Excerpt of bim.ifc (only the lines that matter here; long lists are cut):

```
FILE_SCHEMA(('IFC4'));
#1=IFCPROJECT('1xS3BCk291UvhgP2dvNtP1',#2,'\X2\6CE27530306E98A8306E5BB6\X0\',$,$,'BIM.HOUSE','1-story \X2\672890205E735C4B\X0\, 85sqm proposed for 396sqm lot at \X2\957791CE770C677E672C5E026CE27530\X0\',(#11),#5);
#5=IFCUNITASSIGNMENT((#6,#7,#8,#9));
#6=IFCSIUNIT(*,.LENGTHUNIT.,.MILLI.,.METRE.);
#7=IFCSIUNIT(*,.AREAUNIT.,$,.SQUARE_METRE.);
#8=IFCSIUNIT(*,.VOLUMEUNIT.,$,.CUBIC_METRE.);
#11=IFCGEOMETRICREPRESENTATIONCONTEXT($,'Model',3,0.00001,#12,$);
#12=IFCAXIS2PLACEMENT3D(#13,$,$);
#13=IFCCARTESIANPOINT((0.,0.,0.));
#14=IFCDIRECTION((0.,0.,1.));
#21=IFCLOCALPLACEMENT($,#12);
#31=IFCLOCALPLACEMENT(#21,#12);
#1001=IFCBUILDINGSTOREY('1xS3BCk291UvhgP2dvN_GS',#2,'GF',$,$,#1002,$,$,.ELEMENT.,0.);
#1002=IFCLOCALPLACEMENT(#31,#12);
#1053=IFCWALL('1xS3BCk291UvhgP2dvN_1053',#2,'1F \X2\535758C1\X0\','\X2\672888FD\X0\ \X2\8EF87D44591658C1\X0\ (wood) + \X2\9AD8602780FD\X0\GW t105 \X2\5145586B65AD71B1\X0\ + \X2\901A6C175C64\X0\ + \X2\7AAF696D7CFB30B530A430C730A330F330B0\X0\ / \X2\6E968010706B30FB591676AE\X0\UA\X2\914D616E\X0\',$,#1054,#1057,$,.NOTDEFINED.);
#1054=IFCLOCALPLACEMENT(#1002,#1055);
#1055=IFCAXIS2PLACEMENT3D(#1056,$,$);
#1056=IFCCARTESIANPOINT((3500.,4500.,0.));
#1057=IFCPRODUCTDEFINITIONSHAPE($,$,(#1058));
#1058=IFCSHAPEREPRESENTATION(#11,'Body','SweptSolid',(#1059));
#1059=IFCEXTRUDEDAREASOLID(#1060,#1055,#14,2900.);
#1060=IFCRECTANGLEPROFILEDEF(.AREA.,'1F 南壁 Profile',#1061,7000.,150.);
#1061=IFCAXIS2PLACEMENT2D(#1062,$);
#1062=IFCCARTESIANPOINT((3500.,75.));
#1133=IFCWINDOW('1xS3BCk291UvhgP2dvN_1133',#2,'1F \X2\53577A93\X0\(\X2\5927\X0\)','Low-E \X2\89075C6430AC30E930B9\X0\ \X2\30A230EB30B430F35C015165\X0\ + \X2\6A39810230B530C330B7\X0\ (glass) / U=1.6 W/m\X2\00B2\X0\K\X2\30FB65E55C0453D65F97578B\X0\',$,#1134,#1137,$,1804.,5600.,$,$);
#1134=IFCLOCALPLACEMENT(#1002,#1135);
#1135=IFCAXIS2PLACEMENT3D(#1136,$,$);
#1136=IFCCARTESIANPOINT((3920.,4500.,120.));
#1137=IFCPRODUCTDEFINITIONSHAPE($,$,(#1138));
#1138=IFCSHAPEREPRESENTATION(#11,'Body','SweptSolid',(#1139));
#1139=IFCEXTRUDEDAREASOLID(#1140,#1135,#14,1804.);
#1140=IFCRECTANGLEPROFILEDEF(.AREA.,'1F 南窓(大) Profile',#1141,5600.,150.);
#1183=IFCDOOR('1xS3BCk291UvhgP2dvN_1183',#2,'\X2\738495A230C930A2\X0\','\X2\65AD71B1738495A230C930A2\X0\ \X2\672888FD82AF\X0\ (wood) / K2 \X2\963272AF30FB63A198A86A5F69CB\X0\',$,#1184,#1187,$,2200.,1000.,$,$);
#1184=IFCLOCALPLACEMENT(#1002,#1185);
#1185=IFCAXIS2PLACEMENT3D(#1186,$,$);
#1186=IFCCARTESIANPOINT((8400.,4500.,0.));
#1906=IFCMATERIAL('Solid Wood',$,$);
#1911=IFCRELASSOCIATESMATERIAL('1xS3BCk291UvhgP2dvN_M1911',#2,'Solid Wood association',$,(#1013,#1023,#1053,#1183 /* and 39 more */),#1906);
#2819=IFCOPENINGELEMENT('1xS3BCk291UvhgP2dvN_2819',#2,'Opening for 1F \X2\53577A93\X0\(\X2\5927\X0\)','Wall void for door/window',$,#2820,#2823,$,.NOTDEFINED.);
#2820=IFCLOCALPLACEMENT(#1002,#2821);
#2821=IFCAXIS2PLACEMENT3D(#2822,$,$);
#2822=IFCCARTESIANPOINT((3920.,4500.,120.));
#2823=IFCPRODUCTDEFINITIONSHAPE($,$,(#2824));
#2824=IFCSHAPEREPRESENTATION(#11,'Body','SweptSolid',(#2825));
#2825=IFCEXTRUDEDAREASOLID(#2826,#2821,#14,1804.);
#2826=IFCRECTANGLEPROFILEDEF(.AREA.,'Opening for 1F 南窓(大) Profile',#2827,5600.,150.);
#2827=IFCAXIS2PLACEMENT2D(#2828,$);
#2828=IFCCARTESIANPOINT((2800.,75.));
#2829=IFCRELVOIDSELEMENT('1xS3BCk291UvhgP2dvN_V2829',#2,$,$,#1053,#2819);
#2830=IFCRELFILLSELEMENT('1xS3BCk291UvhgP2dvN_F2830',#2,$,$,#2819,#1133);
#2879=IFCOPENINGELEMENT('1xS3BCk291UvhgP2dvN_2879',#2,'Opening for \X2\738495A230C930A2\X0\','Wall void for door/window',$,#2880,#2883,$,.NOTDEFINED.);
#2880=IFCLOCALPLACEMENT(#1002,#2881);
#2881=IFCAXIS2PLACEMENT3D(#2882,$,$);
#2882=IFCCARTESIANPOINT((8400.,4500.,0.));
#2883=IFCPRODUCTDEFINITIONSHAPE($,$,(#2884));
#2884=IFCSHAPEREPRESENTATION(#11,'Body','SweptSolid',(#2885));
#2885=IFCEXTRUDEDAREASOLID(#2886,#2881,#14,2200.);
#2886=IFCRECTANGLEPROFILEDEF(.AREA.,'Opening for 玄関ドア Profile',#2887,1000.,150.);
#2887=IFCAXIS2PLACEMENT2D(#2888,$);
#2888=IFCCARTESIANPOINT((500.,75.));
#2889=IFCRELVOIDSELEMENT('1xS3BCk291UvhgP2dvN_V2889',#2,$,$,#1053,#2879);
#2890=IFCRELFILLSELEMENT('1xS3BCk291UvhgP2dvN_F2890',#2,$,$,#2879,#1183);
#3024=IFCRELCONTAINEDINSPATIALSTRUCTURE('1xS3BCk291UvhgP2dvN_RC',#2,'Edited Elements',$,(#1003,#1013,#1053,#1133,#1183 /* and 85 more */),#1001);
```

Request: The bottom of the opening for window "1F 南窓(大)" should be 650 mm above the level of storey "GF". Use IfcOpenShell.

```python
import numpy as np
import ifcopenshell
import ifcopenshell.api.geometry
import ifcopenshell.geom
import ifcopenshell.util.element
import ifcopenshell.util.placement
import ifcopenshell.util.shape
import ifcopenshell.util.unit

model = ifcopenshell.open("bim.ifc")
unit_scale = ifcopenshell.util.unit.calculate_unit_scale(model)

window = model.by_guid("1xS3BCk291UvhgP2dvN_1133")
opening = window.FillsVoids[0].RelatingOpeningElement
storey = ifcopenshell.util.element.get_container(window, ifc_class="IfcBuildingStorey")
level = ifcopenshell.util.placement.get_local_placement(storey.ObjectPlacement)[2, 3]

# The opening's origin need not be at the sill, so measure its lowest point.
shape = ifcopenshell.geom.create_shape(ifcopenshell.geom.settings(), opening)
bottom = ifcopenshell.util.shape.get_shape_bottom_elevation(shape, shape.geometry) / unit_scale
dz = level + 0.65 / unit_scale - bottom

shift = np.array([0.0, 0.0, dz])
# The window is not placed relative to its opening, so move both.
for product in (opening, window):
    matrix = ifcopenshell.util.placement.get_local_placement(product.ObjectPlacement)
    matrix[:3, 3] += shift
    ifcopenshell.api.geometry.edit_object_placement(model, product=product, matrix=matrix, is_si=False)

print(f"moved by {dz * unit_scale:+.3f} m")

model.write("bim_v2.ifc")
```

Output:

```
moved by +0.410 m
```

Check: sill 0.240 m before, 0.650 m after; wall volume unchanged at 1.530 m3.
